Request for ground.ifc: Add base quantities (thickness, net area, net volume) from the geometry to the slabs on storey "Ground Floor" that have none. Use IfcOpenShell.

First a look at what the model holds.

```python
import ifcopenshell
import ifcopenshell.util.element
import ifcopenshell.util.unit

model = ifcopenshell.open("ground.ifc")
print(model.schema)
for unit_type in ("LENGTHUNIT", "AREAUNIT", "VOLUMEUNIT"):
    print(unit_type, ifcopenshell.util.unit.calculate_unit_scale(model, unit_type))
storey = next(s for s in model.by_type("IfcBuildingStorey") if s.Name == "Ground Floor")
slabs = [e for e in ifcopenshell.util.element.get_decomposition(storey) if e.is_a("IfcSlab")]
for e in sorted(slabs, key=lambda e: e.id()):
    print(e.id(), e.is_a(), e.Name, list(ifcopenshell.util.element.get_psets(e, qtos_only=True)), sep=" | ")
```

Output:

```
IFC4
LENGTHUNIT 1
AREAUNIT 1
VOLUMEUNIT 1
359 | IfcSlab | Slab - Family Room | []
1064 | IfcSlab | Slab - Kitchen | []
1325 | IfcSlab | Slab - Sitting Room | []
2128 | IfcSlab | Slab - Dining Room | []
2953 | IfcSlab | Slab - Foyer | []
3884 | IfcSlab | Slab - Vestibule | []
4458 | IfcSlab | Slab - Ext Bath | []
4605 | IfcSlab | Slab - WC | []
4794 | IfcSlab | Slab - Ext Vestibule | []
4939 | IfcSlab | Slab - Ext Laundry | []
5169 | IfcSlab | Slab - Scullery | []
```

```python
import ifcopenshell
import ifcopenshell.api.pset
import ifcopenshell.geom
import ifcopenshell.util.element
import ifcopenshell.util.shape
import ifcopenshell.util.unit

model = ifcopenshell.open("ground.ifc")
unit_scale = ifcopenshell.util.unit.calculate_unit_scale(model)
area_scale = ifcopenshell.util.unit.calculate_unit_scale(model, "AREAUNIT")
volume_scale = ifcopenshell.util.unit.calculate_unit_scale(model, "VOLUMEUNIT")
settings = ifcopenshell.geom.settings()

storey = next(s for s in model.by_type("IfcBuildingStorey") if s.Name == "Ground Floor")
slabs = [e for e in ifcopenshell.util.element.get_decomposition(storey) if e.is_a("IfcSlab")]

for e in sorted(slabs, key=lambda e: e.id()):
    if ifcopenshell.util.element.get_psets(e, qtos_only=True, should_inherit=False):
        continue
    # Geometry comes back in metres, in the element's own axes.
    shape = ifcopenshell.geom.create_shape(settings, e)
    values = {
        "Width": ifcopenshell.util.shape.get_z(shape.geometry) / unit_scale,
        "NetArea": ifcopenshell.util.shape.get_footprint_area(shape.geometry) / area_scale,
        "NetVolume": ifcopenshell.util.shape.get_volume(shape.geometry) / volume_scale,
    }
    qto = ifcopenshell.api.pset.add_qto(model, product=e, name="Qto_SlabBaseQuantities")
    ifcopenshell.api.pset.edit_qto(model, qto=qto, properties=values)
    print(e.id(), {k: round(v, 3) for k, v in values.items()})

model.write("ground_rev.ifc")
```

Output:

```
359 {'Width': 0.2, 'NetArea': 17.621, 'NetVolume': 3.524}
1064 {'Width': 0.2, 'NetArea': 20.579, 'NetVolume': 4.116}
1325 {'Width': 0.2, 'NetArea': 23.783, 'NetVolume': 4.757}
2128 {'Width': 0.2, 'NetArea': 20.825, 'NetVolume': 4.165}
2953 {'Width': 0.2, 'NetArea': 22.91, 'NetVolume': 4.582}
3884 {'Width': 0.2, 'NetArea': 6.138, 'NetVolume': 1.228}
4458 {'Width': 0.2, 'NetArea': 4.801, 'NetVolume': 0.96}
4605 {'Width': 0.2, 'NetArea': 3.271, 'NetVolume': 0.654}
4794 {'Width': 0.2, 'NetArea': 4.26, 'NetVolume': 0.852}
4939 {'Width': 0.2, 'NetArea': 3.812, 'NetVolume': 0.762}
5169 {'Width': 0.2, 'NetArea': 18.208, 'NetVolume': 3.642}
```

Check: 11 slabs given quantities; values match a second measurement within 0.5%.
